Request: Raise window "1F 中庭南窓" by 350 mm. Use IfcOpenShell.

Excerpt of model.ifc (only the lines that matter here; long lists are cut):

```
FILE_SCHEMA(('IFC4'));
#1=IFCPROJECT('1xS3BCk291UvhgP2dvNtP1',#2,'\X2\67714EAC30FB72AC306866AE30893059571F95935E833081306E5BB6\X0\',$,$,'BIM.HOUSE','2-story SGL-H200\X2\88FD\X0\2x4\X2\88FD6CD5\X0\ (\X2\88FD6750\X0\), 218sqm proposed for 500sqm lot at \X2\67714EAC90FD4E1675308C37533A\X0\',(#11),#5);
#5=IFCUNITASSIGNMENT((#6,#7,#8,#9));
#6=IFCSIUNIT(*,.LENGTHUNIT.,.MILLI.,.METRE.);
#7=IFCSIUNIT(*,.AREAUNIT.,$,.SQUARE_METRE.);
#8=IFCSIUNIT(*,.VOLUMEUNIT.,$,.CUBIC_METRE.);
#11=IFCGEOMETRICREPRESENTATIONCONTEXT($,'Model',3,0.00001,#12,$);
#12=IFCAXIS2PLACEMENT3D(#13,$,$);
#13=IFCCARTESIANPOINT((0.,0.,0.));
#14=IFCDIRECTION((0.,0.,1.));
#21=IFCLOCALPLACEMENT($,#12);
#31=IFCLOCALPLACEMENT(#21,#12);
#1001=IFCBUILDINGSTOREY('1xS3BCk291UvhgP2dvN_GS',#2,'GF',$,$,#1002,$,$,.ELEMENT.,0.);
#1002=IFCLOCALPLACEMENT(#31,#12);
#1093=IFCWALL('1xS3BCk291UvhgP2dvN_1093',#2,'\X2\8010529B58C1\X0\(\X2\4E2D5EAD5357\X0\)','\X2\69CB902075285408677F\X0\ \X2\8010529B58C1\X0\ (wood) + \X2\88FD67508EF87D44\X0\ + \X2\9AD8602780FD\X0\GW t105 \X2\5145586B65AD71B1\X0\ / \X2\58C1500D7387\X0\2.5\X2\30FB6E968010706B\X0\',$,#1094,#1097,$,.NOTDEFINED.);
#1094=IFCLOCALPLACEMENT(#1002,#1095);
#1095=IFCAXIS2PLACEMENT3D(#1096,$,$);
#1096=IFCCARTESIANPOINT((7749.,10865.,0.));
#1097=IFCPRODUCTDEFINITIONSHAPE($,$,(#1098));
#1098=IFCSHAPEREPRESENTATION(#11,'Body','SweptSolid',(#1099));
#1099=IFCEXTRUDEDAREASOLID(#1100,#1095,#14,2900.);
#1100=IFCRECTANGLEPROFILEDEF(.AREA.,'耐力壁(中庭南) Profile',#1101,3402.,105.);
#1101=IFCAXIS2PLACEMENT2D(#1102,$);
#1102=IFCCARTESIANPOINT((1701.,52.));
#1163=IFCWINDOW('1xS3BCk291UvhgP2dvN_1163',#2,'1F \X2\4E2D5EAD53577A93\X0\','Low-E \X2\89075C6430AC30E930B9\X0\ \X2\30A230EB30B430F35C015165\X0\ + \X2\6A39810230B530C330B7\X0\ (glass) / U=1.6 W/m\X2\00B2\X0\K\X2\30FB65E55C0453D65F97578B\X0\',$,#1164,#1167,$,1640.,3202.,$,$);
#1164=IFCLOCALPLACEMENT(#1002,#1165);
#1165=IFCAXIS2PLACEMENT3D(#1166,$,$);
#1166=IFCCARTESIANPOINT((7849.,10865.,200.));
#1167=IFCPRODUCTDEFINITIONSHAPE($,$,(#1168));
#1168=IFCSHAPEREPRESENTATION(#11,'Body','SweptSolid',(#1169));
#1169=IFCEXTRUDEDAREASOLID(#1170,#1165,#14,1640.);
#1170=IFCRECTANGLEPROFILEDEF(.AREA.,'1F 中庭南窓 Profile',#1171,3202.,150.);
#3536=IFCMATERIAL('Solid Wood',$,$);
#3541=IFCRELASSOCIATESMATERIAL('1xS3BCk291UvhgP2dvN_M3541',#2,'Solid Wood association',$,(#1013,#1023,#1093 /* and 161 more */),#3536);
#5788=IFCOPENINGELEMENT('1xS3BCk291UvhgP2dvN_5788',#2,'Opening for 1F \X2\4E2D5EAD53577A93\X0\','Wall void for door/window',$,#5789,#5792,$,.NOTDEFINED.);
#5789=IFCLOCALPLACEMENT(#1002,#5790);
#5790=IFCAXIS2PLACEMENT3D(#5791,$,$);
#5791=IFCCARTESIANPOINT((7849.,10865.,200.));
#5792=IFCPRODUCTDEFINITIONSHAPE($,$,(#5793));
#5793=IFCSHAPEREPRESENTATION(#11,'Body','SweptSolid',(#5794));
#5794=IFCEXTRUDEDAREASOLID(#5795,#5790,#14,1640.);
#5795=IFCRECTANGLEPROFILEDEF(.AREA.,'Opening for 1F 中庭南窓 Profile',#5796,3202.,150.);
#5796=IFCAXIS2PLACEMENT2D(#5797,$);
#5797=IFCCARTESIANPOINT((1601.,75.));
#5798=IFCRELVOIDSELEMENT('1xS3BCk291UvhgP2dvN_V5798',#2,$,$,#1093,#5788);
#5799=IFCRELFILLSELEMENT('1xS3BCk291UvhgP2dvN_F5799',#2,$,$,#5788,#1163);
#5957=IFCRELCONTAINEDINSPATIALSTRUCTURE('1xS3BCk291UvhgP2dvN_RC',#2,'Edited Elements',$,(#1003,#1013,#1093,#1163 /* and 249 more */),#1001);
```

```python
import numpy as np
import ifcopenshell
import ifcopenshell.api.geometry
import ifcopenshell.util.placement
import ifcopenshell.util.unit

model = ifcopenshell.open("model.ifc")
unit_scale = ifcopenshell.util.unit.calculate_unit_scale(model)

window = model.by_guid("1xS3BCk291UvhgP2dvN_1163")
opening = window.FillsVoids[0].RelatingOpeningElement
dz = 350.0

shift = np.array([0.0, 0.0, dz])
# The window is not placed relative to its opening, so move both.
for product in (opening, window):
    matrix = ifcopenshell.util.placement.get_local_placement(product.ObjectPlacement)
    matrix[:3, 3] += shift
    ifcopenshell.api.geometry.edit_object_placement(model, product=product, matrix=matrix, is_si=False)

print(f"moved by {dz * unit_scale:+.3f} m")

model.write("model_edited.ifc")
```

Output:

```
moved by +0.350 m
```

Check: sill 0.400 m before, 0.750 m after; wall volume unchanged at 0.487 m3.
